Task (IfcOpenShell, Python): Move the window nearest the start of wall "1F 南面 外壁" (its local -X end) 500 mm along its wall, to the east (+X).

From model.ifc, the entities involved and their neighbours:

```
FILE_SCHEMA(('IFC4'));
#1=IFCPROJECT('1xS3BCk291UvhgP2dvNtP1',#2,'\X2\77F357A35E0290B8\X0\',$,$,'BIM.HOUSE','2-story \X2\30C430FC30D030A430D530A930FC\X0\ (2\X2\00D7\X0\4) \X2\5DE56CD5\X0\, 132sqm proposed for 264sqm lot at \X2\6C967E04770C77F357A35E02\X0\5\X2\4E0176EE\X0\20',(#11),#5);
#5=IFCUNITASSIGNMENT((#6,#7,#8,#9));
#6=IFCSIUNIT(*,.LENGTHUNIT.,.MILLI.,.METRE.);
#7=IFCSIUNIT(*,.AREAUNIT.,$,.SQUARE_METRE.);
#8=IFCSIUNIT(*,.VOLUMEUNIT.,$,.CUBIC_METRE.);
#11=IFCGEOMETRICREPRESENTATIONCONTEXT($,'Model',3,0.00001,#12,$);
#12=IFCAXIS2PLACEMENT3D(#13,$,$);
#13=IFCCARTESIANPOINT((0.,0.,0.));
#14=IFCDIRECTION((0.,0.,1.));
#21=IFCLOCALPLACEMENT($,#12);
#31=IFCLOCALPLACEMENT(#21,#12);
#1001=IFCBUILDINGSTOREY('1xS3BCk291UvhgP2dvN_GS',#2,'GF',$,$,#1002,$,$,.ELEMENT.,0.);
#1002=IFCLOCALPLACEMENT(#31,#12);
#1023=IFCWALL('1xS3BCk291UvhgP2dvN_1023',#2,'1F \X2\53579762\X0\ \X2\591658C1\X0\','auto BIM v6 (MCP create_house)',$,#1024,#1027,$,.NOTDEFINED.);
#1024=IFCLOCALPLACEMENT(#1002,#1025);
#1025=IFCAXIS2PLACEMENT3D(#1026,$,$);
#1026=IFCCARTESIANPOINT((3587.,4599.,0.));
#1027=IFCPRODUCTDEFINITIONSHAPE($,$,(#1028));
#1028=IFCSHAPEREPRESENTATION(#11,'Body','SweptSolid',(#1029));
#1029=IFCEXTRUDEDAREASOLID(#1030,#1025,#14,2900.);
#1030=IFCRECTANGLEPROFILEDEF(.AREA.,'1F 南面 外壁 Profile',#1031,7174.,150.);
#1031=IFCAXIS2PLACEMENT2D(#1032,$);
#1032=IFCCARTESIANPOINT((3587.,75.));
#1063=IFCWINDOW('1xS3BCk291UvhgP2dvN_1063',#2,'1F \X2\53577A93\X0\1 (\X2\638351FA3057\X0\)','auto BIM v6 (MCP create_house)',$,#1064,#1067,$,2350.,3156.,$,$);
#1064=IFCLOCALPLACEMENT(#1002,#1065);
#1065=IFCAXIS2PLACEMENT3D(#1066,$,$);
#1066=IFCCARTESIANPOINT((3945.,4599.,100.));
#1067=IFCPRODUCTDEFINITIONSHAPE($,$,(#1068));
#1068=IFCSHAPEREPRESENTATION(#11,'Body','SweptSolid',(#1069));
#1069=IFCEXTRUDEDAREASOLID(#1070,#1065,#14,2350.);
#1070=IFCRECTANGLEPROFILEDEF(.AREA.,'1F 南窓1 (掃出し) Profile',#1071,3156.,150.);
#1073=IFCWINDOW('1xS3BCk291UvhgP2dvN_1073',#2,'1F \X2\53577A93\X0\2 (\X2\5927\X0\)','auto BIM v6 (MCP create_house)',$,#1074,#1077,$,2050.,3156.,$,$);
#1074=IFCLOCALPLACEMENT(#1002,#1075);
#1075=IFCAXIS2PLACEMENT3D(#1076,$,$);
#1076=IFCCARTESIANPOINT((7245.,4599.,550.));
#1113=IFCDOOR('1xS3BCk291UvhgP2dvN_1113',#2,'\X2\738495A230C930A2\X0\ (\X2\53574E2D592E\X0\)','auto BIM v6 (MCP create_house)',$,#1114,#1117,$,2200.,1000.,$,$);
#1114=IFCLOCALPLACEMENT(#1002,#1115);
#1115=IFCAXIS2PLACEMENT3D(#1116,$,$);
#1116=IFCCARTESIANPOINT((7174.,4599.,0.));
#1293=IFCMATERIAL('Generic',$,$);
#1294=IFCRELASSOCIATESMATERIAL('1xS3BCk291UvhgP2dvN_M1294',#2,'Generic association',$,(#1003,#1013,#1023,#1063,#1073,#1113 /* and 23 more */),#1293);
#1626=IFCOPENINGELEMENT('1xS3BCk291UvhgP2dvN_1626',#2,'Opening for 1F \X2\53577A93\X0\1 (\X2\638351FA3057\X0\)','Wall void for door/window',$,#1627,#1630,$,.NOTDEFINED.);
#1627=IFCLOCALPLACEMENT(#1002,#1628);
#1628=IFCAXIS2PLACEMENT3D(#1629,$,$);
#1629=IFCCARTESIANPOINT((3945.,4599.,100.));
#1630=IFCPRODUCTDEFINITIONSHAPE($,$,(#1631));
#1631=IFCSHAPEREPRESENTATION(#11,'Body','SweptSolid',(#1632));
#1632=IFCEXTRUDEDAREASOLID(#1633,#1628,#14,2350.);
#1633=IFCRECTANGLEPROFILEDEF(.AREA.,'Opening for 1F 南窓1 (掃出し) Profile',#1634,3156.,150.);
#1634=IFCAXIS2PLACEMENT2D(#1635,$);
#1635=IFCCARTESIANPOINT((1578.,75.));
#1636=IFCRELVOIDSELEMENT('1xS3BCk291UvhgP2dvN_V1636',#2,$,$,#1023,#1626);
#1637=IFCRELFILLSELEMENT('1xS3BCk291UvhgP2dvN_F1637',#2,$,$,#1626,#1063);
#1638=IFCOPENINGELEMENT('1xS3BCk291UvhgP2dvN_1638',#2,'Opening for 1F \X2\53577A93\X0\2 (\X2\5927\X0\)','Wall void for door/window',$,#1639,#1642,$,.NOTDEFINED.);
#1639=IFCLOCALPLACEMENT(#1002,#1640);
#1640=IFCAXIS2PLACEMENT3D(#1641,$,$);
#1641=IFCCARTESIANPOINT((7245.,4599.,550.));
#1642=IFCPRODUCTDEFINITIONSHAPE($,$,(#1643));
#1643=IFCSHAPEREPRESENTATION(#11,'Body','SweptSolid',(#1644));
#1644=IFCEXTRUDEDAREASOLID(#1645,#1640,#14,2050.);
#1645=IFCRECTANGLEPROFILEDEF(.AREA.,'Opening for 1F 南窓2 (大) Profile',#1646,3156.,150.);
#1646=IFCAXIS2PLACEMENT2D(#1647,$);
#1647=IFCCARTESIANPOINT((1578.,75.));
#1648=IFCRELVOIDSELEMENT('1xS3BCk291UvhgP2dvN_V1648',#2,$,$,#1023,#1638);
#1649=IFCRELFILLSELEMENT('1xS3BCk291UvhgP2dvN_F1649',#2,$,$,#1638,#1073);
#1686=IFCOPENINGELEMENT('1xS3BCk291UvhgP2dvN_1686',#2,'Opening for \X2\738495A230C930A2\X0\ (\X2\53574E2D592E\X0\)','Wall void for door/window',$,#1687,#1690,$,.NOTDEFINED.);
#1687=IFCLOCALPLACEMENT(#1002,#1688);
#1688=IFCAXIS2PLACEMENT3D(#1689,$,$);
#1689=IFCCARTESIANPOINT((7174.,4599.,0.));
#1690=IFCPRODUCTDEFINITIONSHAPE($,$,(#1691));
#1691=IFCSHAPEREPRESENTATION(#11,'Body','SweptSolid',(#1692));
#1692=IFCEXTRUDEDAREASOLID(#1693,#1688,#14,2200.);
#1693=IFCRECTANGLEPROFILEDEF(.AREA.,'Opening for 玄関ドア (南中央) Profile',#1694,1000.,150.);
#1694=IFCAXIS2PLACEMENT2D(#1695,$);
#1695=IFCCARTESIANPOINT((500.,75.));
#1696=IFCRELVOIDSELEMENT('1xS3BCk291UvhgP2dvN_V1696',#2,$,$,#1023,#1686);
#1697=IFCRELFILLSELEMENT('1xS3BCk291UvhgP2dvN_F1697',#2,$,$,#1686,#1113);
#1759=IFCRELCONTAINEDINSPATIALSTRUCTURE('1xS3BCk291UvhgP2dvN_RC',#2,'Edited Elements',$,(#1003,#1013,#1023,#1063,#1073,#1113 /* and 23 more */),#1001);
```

```python
import ifcopenshell
import ifcopenshell.api.geometry
import ifcopenshell.util.placement
import ifcopenshell.util.unit

model = ifcopenshell.open("model.ifc")
unit_scale = ifcopenshell.util.unit.calculate_unit_scale(model)

window = model.by_guid("1xS3BCk291UvhgP2dvN_1063")
opening = window.FillsVoids[0].RelatingOpeningElement
wall = opening.VoidsElements[0].RelatingBuildingElement

wall_matrix = ifcopenshell.util.placement.get_local_placement(wall.ObjectPlacement)
shift = wall_matrix[:3, 0] * 0.5 / unit_scale
before = ifcopenshell.util.placement.get_local_placement(window.ObjectPlacement)[:3, 3].copy()

# The window is not placed relative to its opening, so move both.
for product in (opening, window):
    matrix = ifcopenshell.util.placement.get_local_placement(product.ObjectPlacement)
    matrix[:3, 3] += shift
    ifcopenshell.api.geometry.edit_object_placement(model, product=product, matrix=matrix, is_si=False)

after = ifcopenshell.util.placement.get_local_placement(window.ObjectPlacement)[:3, 3]
print("window moved by", (after - before).round(3) + 0.0)

model.write("model_rev.ifc")
```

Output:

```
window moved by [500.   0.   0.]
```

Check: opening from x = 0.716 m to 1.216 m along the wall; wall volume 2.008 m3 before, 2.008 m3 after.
